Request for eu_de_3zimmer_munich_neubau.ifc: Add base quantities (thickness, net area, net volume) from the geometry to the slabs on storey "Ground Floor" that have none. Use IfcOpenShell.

First a look at what the model holds.

```python
import ifcopenshell
import ifcopenshell.util.element
import ifcopenshell.util.unit

model = ifcopenshell.open("eu_de_3zimmer_munich_neubau.ifc")
print(model.schema)
for unit_type in ("LENGTHUNIT", "AREAUNIT", "VOLUMEUNIT"):
    print(unit_type, ifcopenshell.util.unit.calculate_unit_scale(model, unit_type))
storey = next(s for s in model.by_type("IfcBuildingStorey") if s.Name == "Ground Floor")
slabs = [e for e in ifcopenshell.util.element.get_decomposition(storey) if e.is_a("IfcSlab")]
for e in sorted(slabs, key=lambda e: e.id()):
    print(e.id(), e.is_a(), e.Name, list(ifcopenshell.util.element.get_psets(e, qtos_only=True)), sep=" | ")
```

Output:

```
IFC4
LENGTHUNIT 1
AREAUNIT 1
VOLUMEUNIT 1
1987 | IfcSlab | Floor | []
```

```python
import ifcopenshell
import ifcopenshell.api.pset
import ifcopenshell.geom
import ifcopenshell.util.element
import ifcopenshell.util.shape
import ifcopenshell.util.unit

model = ifcopenshell.open("eu_de_3zimmer_munich_neubau.ifc")
unit_scale = ifcopenshell.util.unit.calculate_unit_scale(model)
area_scale = ifcopenshell.util.unit.calculate_unit_scale(model, "AREAUNIT")
volume_scale = ifcopenshell.util.unit.calculate_unit_scale(model, "VOLUMEUNIT")
settings = ifcopenshell.geom.settings()

storey = next(s for s in model.by_type("IfcBuildingStorey") if s.Name == "Ground Floor")
slabs = [e for e in ifcopenshell.util.element.get_decomposition(storey) if e.is_a("IfcSlab")]

for e in sorted(slabs, key=lambda e: e.id()):
    if ifcopenshell.util.element.get_psets(e, qtos_only=True, should_inherit=False):
        continue
    # Geometry comes back in metres, in the element's own axes.
    shape = ifcopenshell.geom.create_shape(settings, e)
    values = {
        "Width": ifcopenshell.util.shape.get_z(shape.geometry) / unit_scale,
        "NetArea": ifcopenshell.util.shape.get_footprint_area(shape.geometry) / area_scale,
        "NetVolume": ifcopenshell.util.shape.get_volume(shape.geometry) / volume_scale,
    }
    qto = ifcopenshell.api.pset.add_qto(model, product=e, name="Qto_SlabBaseQuantities")
    ifcopenshell.api.pset.edit_qto(model, qto=qto, properties=values)
    print(e.id(), {k: round(v, 3) for k, v in values.items()})

model.write("eu_de_3zimmer_munich_neubau_updated.ifc")
```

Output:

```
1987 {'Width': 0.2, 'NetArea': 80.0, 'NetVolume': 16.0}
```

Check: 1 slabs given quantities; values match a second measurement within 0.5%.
